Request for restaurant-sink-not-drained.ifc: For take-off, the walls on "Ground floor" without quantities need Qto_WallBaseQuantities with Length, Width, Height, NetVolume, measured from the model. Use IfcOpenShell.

First a look at what the model holds.

```python
import ifcopenshell
import ifcopenshell.util.element
import ifcopenshell.util.unit

model = ifcopenshell.open("restaurant-sink-not-drained.ifc")
print(model.schema)
for unit_type in ("LENGTHUNIT", "AREAUNIT", "VOLUMEUNIT"):
    print(unit_type, ifcopenshell.util.unit.calculate_unit_scale(model, unit_type))
storey = next(s for s in model.by_type("IfcBuildingStorey") if s.Name == "Ground floor")
walls = [e for e in ifcopenshell.util.element.get_decomposition(storey) if e.is_a("IfcWall")]
for e in sorted(walls, key=lambda e: e.id()):
    print(e.id(), e.is_a(), e.Name, list(ifcopenshell.util.element.get_psets(e, qtos_only=True)), sep=" | ")
```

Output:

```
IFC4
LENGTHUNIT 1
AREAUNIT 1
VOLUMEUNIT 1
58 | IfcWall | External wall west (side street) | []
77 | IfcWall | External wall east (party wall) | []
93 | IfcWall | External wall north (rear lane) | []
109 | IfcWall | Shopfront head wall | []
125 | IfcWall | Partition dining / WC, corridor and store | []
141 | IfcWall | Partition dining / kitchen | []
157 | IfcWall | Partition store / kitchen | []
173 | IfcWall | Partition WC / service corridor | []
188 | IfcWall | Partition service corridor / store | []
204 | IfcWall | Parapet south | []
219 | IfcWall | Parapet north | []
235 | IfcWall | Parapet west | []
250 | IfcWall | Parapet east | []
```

```python
import ifcopenshell
import ifcopenshell.api.pset
import ifcopenshell.geom
import ifcopenshell.util.element
import ifcopenshell.util.shape
import ifcopenshell.util.unit

model = ifcopenshell.open("restaurant-sink-not-drained.ifc")
unit_scale = ifcopenshell.util.unit.calculate_unit_scale(model)
volume_scale = ifcopenshell.util.unit.calculate_unit_scale(model, "VOLUMEUNIT")
settings = ifcopenshell.geom.settings()

storey = next(s for s in model.by_type("IfcBuildingStorey") if s.Name == "Ground floor")
walls = [e for e in ifcopenshell.util.element.get_decomposition(storey) if e.is_a("IfcWall")]

for e in sorted(walls, key=lambda e: e.id()):
    if ifcopenshell.util.element.get_psets(e, qtos_only=True, should_inherit=False):
        continue
    # Geometry comes back in metres, in the element's own axes.
    shape = ifcopenshell.geom.create_shape(settings, e)
    values = {
        "Length": ifcopenshell.util.shape.get_x(shape.geometry) / unit_scale,
        "Width": ifcopenshell.util.shape.get_y(shape.geometry) / unit_scale,
        "Height": ifcopenshell.util.shape.get_z(shape.geometry) / unit_scale,
        "NetVolume": ifcopenshell.util.shape.get_volume(shape.geometry) / volume_scale,
    }
    qto = ifcopenshell.api.pset.add_qto(model, product=e, name="Qto_WallBaseQuantities")
    ifcopenshell.api.pset.edit_qto(model, qto=qto, properties=values)
    print(e.id(), {k: round(v, 3) for k, v in values.items()})

model.write("restaurant-sink-not-drained_v2.ifc")
```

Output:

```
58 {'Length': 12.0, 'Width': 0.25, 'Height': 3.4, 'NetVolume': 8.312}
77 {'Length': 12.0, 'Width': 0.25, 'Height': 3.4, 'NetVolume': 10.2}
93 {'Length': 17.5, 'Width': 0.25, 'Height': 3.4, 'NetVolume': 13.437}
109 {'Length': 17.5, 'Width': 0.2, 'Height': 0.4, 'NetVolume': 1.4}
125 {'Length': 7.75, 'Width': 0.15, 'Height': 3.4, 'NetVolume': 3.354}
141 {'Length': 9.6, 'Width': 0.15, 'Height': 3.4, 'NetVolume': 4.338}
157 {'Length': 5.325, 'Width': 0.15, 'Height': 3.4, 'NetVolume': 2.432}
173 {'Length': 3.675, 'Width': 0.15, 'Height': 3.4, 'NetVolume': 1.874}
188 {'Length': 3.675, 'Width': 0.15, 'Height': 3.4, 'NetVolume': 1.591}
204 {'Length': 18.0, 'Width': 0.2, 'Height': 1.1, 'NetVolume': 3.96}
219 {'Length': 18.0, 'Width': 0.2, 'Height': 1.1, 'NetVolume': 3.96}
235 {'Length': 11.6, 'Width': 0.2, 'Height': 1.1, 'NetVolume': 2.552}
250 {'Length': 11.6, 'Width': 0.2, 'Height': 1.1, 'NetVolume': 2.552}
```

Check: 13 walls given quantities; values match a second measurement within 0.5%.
